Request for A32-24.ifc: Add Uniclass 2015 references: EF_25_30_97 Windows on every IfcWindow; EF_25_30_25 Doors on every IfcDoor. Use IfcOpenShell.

First a look at what the model holds.

```python
import ifcopenshell

model = ifcopenshell.open("A32-24.ifc")
print(model.schema)
print("classifications:", [c.Name for c in model.by_type("IfcClassification")])
for ifc_class in ("IfcDoor", "IfcRoof", "IfcStair", "IfcWall", "IfcWindow"):
    print(ifc_class, len(model.by_type(ifc_class)))
```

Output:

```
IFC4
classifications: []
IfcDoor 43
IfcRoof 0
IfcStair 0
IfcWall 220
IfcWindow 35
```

```python
import ifcopenshell
import ifcopenshell.api.classification

model = ifcopenshell.open("A32-24.ifc")

system = ifcopenshell.api.classification.add_classification(model, classification="Uniclass 2015")

codes = {
    "IfcWindow": ("EF_25_30_97", "Windows"),
    "IfcDoor": ("EF_25_30_25", "Doors"),
}
for ifc_class, (code, name) in codes.items():
    products = model.by_type(ifc_class)
    ifcopenshell.api.classification.add_reference(
        model, products=products, classification=system, identification=code, name=name
    )
    print(code, len(products))

model.write("A32-24_edited.ifc")
```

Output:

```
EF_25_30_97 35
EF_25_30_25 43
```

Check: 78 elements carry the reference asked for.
